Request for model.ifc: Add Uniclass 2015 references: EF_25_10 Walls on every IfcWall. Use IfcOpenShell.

First a look at what the model holds.

```python
import ifcopenshell

model = ifcopenshell.open("model.ifc")
print(model.schema)
print("classifications:", [c.Name for c in model.by_type("IfcClassification")])
for ifc_class in ("IfcDoor", "IfcRoof", "IfcStair", "IfcWall", "IfcWindow"):
    print(ifc_class, len(model.by_type(ifc_class)))
```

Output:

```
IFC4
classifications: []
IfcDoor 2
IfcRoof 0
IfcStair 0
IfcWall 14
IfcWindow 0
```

```python
import ifcopenshell
import ifcopenshell.api.classification

model = ifcopenshell.open("model.ifc")

system = ifcopenshell.api.classification.add_classification(model, classification="Uniclass 2015")

codes = {
    "IfcWall": ("EF_25_10", "Walls"),
}
for ifc_class, (code, name) in codes.items():
    products = model.by_type(ifc_class)
    ifcopenshell.api.classification.add_reference(
        model, products=products, classification=system, identification=code, name=name
    )
    print(code, len(products))

model.write("model-out.ifc")
```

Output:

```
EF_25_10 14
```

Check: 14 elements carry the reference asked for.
